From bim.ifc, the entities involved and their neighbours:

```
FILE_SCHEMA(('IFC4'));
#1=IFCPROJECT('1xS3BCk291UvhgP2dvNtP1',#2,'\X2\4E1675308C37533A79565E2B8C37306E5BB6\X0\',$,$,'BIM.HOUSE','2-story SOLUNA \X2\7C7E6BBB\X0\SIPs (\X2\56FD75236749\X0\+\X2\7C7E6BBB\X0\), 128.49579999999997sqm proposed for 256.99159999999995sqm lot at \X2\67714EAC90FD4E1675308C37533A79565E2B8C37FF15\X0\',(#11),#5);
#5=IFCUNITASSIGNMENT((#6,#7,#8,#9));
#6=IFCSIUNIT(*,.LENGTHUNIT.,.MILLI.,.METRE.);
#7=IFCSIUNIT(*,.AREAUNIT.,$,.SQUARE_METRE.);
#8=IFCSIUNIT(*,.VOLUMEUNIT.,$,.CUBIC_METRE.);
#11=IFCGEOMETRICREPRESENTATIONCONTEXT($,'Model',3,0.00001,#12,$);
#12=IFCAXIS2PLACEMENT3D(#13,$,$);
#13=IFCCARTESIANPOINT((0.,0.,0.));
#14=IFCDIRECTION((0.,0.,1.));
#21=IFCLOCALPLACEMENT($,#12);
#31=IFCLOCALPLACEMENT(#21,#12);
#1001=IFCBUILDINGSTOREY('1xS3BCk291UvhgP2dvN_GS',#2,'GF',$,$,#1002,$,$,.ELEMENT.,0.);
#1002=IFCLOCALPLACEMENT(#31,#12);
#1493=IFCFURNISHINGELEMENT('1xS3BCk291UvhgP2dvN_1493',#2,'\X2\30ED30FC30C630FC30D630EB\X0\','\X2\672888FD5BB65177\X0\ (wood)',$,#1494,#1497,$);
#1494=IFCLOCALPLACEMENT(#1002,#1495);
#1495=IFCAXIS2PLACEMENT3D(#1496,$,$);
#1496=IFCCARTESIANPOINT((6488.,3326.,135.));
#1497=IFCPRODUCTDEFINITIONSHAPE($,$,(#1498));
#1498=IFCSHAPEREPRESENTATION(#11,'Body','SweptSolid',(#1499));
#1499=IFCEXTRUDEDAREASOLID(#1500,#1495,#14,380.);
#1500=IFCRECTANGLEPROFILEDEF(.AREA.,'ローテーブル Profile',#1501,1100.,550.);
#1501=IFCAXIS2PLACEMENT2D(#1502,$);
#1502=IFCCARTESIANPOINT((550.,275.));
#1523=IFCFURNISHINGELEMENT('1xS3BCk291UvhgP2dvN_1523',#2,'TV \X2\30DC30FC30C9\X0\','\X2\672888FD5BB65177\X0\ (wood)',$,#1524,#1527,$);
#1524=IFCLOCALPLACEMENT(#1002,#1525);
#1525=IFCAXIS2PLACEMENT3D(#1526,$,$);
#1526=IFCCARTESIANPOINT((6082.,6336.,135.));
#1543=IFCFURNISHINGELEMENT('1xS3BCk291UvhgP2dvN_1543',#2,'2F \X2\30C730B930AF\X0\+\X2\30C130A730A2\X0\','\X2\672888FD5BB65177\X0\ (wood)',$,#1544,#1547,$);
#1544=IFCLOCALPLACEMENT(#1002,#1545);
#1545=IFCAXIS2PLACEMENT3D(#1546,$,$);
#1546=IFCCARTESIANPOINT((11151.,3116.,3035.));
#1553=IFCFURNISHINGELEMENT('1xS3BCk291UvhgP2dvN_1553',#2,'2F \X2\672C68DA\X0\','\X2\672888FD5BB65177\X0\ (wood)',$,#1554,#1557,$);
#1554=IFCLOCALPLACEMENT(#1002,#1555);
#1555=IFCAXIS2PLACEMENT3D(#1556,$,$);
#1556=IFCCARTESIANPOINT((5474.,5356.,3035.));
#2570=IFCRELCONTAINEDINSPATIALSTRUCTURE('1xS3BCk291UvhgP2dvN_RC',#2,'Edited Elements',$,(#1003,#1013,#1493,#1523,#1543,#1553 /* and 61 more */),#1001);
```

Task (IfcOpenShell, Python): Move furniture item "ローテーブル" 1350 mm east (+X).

```python
import ifcopenshell
import ifcopenshell.api.geometry
import ifcopenshell.util.placement
import ifcopenshell.util.unit

model = ifcopenshell.open("bim.ifc")
unit_scale = ifcopenshell.util.unit.calculate_unit_scale(model)

item = model.by_guid("1xS3BCk291UvhgP2dvN_1493")
matrix = ifcopenshell.util.placement.get_local_placement(item.ObjectPlacement)
matrix[0, 3] += 1.35 / unit_scale
ifcopenshell.api.geometry.edit_object_placement(model, product=item, matrix=matrix, is_si=False)

print(ifcopenshell.util.placement.get_local_placement(item.ObjectPlacement).round(3) + 0.0)

model.write("bim-out.ifc")
```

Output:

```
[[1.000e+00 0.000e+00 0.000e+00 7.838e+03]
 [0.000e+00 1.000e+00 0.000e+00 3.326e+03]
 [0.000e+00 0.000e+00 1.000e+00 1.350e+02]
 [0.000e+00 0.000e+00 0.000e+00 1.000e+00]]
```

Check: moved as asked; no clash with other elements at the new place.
